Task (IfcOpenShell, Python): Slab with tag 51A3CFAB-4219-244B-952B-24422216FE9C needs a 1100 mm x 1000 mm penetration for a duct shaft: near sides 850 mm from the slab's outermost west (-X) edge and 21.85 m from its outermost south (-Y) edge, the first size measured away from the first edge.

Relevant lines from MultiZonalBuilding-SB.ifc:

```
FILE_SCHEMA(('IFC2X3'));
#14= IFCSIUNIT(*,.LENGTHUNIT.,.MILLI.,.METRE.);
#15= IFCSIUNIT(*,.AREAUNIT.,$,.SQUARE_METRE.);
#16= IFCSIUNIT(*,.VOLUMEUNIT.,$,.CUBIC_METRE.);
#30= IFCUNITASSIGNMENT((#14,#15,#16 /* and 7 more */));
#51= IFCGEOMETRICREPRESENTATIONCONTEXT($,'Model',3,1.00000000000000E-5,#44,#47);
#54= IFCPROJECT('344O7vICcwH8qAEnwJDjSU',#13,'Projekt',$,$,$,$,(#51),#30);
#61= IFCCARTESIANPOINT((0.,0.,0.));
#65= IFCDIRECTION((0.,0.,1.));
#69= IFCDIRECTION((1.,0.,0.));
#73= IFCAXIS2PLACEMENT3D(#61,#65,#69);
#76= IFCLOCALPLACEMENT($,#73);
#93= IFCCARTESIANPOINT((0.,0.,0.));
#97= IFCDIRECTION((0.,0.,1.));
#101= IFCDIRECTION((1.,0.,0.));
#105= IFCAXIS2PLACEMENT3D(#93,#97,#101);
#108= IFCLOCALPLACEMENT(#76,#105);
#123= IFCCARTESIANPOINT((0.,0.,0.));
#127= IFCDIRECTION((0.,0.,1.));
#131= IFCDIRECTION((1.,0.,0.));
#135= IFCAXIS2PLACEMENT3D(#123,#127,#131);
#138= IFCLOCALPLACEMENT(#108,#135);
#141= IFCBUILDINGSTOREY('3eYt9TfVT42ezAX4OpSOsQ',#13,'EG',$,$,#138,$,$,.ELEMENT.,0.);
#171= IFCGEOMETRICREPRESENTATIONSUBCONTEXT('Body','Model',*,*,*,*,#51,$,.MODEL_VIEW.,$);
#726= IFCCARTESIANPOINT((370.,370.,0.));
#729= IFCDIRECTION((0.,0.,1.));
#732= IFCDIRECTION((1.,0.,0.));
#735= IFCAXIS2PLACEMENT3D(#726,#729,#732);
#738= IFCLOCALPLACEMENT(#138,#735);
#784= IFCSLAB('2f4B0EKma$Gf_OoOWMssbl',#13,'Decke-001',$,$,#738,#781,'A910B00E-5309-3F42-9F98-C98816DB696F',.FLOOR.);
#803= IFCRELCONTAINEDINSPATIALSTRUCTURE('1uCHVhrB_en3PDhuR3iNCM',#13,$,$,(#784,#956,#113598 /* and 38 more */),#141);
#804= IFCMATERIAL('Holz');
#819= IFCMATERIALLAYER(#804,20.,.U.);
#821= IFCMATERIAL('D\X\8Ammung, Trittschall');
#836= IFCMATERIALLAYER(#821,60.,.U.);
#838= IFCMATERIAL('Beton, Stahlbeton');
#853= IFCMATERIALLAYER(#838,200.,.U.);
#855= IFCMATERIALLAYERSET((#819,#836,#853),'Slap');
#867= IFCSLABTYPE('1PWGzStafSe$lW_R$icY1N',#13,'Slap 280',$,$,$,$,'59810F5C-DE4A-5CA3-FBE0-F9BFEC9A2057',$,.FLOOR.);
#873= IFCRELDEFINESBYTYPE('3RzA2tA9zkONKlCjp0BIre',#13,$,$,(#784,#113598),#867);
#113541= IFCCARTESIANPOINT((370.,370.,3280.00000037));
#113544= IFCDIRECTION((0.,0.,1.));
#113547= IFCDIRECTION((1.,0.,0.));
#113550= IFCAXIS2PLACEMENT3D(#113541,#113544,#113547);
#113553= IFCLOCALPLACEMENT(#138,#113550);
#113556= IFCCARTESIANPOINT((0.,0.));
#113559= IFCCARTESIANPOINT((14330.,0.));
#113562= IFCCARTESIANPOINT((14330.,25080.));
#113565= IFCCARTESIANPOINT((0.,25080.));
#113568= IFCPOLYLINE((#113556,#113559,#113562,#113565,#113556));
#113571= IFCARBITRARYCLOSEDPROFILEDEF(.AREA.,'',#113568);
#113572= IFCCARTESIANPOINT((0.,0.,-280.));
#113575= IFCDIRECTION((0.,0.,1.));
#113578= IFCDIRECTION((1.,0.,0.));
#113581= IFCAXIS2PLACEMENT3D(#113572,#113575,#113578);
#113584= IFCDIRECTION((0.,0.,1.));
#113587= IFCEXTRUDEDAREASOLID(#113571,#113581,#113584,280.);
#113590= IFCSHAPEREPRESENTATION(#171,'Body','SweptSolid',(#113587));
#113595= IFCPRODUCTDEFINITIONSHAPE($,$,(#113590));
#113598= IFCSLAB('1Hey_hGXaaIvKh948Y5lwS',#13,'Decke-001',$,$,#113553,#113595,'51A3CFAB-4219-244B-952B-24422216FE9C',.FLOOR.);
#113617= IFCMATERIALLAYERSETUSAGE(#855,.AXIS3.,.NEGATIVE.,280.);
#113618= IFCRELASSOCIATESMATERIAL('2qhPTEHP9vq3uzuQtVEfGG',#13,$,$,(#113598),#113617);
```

```python
import numpy as np
import ifcopenshell
import ifcopenshell.api.feature
import ifcopenshell.api.geometry
import ifcopenshell.api.root
import ifcopenshell.geom
import ifcopenshell.util.placement
import ifcopenshell.util.representation
import ifcopenshell.util.shape
import ifcopenshell.util.unit

model = ifcopenshell.open("MultiZonalBuilding-SB.ifc")
unit_scale = ifcopenshell.util.unit.calculate_unit_scale(model)
settings = ifcopenshell.geom.settings()


def volume(element):
    """Net volume in cubic metres, openings subtracted."""
    shape = ifcopenshell.geom.create_shape(settings, element)
    return ifcopenshell.util.shape.get_volume(shape.geometry)


slab = model.by_id(113598)
before = volume(slab)

# Extent in the slab's own axes, in metres. The edges named are its -X and -Y sides.
slab_shape = ifcopenshell.geom.create_shape(settings, slab)
vertices = ifcopenshell.util.shape.get_vertices(slab_shape.geometry)
x_min, y_min, bottom = vertices.min(axis=0)
top = vertices[:, 2].max()

opening = ifcopenshell.api.root.create_entity(model, ifc_class="IfcOpeningElement", name="Duct shaft opening")
context = ifcopenshell.util.representation.get_context(model, "Model", "Body", "MODEL_VIEW")
width, depth = 1.1, 1
outline = [(0.0, 0.0), (width, 0.0), (width, depth), (0.0, depth), (0.0, 0.0)]
# Overshoot both faces by 50 mm so the cut is clean.
shape = ifcopenshell.api.geometry.add_slab_representation(
    model, context=context, depth=top - bottom + 0.1, polyline=outline
)
ifcopenshell.api.geometry.assign_representation(model, product=opening, representation=shape)

matrix = ifcopenshell.util.placement.get_local_placement(slab.ObjectPlacement)
matrix[:, 3] = matrix @ np.append(np.array([x_min + 0.85, y_min + 21.85, bottom - 0.05]) / unit_scale, 1.0)
ifcopenshell.api.geometry.edit_object_placement(model, product=opening, matrix=matrix, is_si=False)
ifcopenshell.api.feature.add_feature(model, feature=opening, element=slab)

after = volume(slab)

print(f"slab volume {before:.3f} -> {after:.3f} m3")

model.write("MultiZonalBuilding-SB_edited.ifc")
```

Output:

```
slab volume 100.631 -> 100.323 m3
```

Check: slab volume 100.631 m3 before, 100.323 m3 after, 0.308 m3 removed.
